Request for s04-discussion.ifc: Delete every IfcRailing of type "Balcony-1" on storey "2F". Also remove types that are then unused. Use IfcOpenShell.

First a look at what the model holds.

```python
import ifcopenshell
import ifcopenshell.util.element

model = ifcopenshell.open("s04-discussion.ifc")
print(model.schema)
storey = next(s for s in model.by_type("IfcBuildingStorey") if s.Name == "2F")
railings = [e for e in ifcopenshell.util.element.get_decomposition(storey) if e.is_a("IfcRailing")]
seen = {}
for e in railings:
    element_type = ifcopenshell.util.element.get_type(e)
    name = element_type.Name if element_type not in (None, e) else None
    seen[name] = seen.get(name, 0) + 1
for name, count in sorted(seen.items(), key=str):
    print(count, "x", name)
```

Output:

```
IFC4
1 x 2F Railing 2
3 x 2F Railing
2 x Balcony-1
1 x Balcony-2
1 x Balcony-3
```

```python
import ifcopenshell
import ifcopenshell.api.root
import ifcopenshell.util.element

model = ifcopenshell.open("s04-discussion.ifc")

storey = next(s for s in model.by_type("IfcBuildingStorey") if s.Name == "2F")
railings = [e for e in ifcopenshell.util.element.get_decomposition(storey) if e.is_a("IfcRailing")]
targets = [e for e in railings if (t := ifcopenshell.util.element.get_type(e)) not in (None, e) and t.Name == "Balcony-1"]
types = {ifcopenshell.util.element.get_type(e) for e in targets} - {None, *targets}

for e in targets:
    ifcopenshell.api.root.remove_product(model, product=e)
print(len(targets), "removed")

unused = [t for t in types if not ifcopenshell.util.element.get_types(t)]
for t in unused:
    ifcopenshell.api.root.remove_product(model, product=t)
print(len(unused), "unused types removed")

model.write("s04-discussion_updated.ifc")
```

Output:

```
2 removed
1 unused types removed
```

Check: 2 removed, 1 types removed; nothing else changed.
